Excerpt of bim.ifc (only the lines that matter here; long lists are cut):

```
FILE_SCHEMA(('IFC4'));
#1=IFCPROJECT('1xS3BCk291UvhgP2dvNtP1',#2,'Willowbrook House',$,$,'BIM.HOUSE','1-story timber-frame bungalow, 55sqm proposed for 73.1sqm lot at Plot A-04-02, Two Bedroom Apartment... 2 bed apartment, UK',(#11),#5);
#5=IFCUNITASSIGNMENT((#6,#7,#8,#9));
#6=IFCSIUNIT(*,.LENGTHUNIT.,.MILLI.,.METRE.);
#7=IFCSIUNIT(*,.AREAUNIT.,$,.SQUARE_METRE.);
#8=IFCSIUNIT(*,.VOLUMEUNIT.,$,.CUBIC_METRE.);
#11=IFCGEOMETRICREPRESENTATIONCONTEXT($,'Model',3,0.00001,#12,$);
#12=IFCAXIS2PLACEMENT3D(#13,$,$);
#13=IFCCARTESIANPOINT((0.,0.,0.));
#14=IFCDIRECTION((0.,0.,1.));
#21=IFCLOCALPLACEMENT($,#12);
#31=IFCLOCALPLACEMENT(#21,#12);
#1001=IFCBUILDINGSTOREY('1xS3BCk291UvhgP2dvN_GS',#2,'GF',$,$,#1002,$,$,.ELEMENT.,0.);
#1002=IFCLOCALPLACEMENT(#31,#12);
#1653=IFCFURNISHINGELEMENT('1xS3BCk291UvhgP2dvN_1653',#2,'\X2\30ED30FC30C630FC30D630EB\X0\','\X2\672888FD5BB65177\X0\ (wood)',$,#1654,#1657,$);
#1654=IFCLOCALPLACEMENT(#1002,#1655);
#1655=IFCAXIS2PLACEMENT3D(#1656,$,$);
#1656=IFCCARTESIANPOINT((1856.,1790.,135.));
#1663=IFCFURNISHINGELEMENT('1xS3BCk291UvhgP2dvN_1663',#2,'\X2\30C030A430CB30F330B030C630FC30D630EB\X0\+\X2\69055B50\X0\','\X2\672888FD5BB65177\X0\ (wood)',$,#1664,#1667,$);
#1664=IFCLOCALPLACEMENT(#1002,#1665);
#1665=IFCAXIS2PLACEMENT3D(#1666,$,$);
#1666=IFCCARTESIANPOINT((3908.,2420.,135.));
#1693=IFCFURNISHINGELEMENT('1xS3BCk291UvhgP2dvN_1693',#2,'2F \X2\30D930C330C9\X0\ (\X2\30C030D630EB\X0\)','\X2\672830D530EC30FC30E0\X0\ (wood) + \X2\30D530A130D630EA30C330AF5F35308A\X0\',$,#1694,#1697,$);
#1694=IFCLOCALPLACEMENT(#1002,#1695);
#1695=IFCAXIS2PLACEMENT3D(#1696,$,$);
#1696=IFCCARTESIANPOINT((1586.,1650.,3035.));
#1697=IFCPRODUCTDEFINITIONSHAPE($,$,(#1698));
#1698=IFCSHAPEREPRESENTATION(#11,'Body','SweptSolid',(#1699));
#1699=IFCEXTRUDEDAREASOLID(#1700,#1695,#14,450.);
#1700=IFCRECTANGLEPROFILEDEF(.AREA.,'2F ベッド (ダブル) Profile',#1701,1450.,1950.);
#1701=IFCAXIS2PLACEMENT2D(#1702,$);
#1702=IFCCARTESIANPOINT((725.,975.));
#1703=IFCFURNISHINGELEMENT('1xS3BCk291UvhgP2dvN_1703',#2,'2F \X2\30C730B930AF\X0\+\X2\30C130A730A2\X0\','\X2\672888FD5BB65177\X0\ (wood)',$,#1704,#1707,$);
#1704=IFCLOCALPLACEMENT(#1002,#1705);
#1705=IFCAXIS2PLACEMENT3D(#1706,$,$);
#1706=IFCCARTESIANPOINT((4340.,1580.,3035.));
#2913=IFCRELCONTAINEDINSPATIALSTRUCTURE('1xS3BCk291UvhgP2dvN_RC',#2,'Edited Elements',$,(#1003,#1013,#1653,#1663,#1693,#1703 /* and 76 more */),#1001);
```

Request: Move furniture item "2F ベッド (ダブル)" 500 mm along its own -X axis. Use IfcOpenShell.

```python
import ifcopenshell
import ifcopenshell.api.geometry
import ifcopenshell.util.placement

model = ifcopenshell.open("bim.ifc")

item = model.by_id(1693)
matrix = ifcopenshell.util.placement.get_local_placement(item.ObjectPlacement)
matrix[:3, 3] -= matrix[:3, 0] * 500.0
ifcopenshell.api.geometry.edit_object_placement(model, product=item, matrix=matrix, is_si=False)

print(ifcopenshell.util.placement.get_local_placement(item.ObjectPlacement).round(3) + 0.0)

model.write("bim-out.ifc")
```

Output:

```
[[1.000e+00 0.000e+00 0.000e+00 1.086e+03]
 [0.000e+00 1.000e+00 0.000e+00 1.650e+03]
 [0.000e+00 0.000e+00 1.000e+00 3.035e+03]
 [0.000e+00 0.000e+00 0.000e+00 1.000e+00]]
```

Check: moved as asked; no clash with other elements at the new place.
